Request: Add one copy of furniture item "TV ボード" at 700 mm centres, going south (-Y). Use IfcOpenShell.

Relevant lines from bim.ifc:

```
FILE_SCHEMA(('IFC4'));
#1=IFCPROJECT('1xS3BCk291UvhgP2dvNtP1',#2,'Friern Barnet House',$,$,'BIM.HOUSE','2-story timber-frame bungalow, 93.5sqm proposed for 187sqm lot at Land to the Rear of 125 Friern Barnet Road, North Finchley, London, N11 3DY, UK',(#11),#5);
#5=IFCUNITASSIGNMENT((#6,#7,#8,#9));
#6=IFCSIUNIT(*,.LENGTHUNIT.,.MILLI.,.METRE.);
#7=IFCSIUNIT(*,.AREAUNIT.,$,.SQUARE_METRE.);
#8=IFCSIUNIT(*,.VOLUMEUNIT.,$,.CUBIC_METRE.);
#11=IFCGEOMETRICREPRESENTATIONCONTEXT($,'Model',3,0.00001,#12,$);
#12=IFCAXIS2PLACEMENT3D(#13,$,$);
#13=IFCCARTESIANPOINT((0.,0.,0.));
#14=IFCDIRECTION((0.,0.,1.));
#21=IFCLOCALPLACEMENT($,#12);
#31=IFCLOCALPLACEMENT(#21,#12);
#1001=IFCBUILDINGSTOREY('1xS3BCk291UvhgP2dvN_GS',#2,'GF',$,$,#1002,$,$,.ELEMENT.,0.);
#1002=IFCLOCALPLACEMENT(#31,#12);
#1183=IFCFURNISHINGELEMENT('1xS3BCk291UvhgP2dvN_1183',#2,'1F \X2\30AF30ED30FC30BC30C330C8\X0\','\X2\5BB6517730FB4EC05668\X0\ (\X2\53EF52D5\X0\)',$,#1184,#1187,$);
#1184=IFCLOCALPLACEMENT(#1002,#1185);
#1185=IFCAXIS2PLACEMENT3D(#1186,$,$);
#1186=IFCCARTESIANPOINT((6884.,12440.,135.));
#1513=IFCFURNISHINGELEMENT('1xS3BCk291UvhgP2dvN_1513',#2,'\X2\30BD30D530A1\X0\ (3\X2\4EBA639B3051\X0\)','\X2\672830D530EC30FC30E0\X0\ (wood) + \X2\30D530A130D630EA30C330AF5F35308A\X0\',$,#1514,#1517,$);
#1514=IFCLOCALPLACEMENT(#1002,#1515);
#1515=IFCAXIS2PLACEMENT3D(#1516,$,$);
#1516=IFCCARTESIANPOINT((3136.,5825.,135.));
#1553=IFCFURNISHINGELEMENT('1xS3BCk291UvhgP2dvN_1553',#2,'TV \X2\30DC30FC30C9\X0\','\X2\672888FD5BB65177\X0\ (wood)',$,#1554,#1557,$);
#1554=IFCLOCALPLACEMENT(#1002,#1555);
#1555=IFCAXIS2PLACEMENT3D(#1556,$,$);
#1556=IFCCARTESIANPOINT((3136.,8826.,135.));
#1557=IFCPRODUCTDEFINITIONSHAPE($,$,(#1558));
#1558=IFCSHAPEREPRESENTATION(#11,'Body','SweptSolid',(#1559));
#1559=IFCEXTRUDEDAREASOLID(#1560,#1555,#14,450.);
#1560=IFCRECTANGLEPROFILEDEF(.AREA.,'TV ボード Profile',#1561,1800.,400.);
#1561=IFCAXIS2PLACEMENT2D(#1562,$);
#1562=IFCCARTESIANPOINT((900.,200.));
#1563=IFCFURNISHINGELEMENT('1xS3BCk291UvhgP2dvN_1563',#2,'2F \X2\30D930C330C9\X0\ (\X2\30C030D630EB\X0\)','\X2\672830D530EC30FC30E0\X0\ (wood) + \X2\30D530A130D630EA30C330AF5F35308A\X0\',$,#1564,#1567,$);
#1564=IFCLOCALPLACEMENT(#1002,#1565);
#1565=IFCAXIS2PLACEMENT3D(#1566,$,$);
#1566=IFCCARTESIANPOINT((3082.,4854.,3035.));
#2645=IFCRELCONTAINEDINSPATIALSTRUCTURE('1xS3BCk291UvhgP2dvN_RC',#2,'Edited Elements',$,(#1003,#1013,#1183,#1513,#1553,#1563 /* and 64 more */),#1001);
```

```python
import numpy as np
import ifcopenshell
import ifcopenshell.api.geometry
import ifcopenshell.api.root
import ifcopenshell.util.element
import ifcopenshell.util.placement

model = ifcopenshell.open("bim.ifc")


def reuse_history(source, copy):
    """copy_class also copies each property set's owner history, people and application; keep the originals."""
    for rel in copy.IsDefinedBy:
        if rel.is_a("IfcRelDefinesByProperties") and (history := rel.RelatingPropertyDefinition.OwnerHistory):
            rel.RelatingPropertyDefinition.OwnerHistory = source.OwnerHistory
            ifcopenshell.util.element.remove_deep2(model, history)


source = model.by_guid("1xS3BCk291UvhgP2dvN_1553")
base = ifcopenshell.util.placement.get_local_placement(source.ObjectPlacement)
step = np.array([0.0, -1.0, 0.0]) * 700.0

for i in range(1, 2):
    copy = ifcopenshell.api.root.copy_class(model, product=source)
    copy.Representation = ifcopenshell.util.element.copy_deep(
        model, source.Representation, exclude=["IfcGeometricRepresentationContext", "IfcRepresentationMap"]
    )
    reuse_history(source, copy)
    matrix = base.copy()
    matrix[:3, 3] += i * step
    print("added at", matrix[:3, 3].round(3) + 0.0)
    ifcopenshell.api.geometry.edit_object_placement(model, product=copy, matrix=matrix, is_si=False)

model.write("bim_v2.ifc")
```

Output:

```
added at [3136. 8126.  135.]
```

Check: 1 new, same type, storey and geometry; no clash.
